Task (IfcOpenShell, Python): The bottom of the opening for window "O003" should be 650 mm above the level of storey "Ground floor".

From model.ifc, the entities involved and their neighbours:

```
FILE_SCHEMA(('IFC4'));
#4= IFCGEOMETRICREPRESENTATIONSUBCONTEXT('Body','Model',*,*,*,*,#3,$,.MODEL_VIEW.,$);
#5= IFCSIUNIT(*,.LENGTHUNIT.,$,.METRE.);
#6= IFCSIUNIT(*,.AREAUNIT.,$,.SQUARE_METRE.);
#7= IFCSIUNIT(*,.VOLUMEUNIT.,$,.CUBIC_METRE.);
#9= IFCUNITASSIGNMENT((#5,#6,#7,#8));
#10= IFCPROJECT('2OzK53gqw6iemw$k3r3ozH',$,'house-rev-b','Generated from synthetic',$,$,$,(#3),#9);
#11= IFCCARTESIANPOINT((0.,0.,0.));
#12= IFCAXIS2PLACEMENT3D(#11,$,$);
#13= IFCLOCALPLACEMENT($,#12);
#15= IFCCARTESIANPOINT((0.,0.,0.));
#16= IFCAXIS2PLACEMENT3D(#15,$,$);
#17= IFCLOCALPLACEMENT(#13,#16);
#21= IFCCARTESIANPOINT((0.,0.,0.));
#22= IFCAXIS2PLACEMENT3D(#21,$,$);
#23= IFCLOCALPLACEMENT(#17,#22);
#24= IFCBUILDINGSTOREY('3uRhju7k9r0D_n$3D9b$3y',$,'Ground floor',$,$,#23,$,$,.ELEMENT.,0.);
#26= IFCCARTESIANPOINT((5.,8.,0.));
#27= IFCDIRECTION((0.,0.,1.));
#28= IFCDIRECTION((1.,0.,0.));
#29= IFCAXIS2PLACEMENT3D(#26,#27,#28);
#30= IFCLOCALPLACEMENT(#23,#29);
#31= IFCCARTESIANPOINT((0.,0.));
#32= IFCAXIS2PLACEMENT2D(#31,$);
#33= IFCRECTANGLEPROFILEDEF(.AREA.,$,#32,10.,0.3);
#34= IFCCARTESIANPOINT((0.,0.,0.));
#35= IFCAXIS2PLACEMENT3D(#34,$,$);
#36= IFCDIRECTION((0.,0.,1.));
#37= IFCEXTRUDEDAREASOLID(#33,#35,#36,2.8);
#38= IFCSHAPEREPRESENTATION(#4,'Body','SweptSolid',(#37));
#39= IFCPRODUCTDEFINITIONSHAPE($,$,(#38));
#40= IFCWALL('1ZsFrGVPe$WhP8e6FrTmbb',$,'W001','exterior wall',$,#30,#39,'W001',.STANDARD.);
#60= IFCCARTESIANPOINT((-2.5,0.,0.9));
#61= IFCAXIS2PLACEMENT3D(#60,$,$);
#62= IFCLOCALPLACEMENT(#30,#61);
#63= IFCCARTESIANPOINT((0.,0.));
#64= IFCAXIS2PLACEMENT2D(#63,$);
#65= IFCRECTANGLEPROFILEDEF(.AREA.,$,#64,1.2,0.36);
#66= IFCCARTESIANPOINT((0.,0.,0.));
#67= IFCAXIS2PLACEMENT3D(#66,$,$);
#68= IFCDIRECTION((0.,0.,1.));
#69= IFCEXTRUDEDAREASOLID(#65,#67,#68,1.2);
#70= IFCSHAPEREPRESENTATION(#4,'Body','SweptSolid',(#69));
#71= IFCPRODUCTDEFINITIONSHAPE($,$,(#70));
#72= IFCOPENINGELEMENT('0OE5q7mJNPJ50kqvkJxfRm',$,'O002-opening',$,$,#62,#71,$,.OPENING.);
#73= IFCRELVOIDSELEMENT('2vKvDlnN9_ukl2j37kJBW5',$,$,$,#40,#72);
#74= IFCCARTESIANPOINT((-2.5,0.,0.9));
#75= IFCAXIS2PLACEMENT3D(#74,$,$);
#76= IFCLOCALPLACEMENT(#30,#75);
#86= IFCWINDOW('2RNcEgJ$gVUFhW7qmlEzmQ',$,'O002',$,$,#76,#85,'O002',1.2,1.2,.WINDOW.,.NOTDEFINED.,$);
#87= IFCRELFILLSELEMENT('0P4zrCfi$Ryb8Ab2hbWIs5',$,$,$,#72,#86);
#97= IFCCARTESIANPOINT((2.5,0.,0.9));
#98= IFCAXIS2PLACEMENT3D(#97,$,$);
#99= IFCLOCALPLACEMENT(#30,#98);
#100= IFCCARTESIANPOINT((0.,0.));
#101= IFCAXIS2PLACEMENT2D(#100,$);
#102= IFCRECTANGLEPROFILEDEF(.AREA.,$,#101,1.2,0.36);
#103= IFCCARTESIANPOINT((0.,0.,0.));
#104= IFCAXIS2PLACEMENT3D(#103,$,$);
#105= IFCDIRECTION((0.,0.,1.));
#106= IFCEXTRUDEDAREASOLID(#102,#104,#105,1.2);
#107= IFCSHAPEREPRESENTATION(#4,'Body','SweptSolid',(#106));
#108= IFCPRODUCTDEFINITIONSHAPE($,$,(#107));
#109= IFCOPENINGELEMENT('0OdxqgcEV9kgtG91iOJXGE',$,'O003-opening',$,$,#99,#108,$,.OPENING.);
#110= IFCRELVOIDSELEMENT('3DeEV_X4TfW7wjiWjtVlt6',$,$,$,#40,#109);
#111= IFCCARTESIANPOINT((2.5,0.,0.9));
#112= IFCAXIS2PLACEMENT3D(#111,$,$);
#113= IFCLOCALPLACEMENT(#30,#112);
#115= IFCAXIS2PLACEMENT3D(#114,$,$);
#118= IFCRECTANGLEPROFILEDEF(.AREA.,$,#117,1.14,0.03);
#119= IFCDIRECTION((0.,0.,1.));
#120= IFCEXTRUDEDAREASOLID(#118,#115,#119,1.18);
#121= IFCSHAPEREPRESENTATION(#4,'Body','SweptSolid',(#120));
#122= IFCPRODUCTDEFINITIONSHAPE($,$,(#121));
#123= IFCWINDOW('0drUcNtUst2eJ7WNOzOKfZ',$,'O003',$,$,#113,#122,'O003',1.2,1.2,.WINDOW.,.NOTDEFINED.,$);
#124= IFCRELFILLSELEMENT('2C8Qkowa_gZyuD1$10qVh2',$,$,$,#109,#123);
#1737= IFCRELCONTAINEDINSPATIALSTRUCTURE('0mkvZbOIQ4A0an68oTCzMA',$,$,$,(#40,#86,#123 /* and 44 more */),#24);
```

```python
import numpy as np
import ifcopenshell
import ifcopenshell.api.geometry
import ifcopenshell.geom
import ifcopenshell.util.element
import ifcopenshell.util.placement
import ifcopenshell.util.shape
import ifcopenshell.util.unit

model = ifcopenshell.open("model.ifc")
unit_scale = ifcopenshell.util.unit.calculate_unit_scale(model)

window = model.by_id(123)
opening = window.FillsVoids[0].RelatingOpeningElement
storey = ifcopenshell.util.element.get_container(window, ifc_class="IfcBuildingStorey")
level = ifcopenshell.util.placement.get_local_placement(storey.ObjectPlacement)[2, 3]

# The opening's origin need not be at the sill, so measure its lowest point.
shape = ifcopenshell.geom.create_shape(ifcopenshell.geom.settings(), opening)
bottom = ifcopenshell.util.shape.get_shape_bottom_elevation(shape, shape.geometry) / unit_scale
dz = level + 0.65 / unit_scale - bottom

shift = np.array([0.0, 0.0, dz])
# The window is not placed relative to its opening, so move both.
for product in (opening, window):
    matrix = ifcopenshell.util.placement.get_local_placement(product.ObjectPlacement)
    matrix[:3, 3] += shift
    ifcopenshell.api.geometry.edit_object_placement(model, product=product, matrix=matrix, is_si=False)

print(f"moved by {dz * unit_scale:+.3f} m")

model.write("model_edited.ifc")
```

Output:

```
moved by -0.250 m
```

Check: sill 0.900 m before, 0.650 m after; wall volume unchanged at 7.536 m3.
